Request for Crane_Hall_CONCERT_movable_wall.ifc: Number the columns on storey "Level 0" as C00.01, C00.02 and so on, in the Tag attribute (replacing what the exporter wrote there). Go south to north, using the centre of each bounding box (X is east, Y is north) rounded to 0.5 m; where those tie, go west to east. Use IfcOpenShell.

First a look at what the model holds.

```python
import ifcopenshell
import ifcopenshell.util.element
import ifcopenshell.util.placement

model = ifcopenshell.open("Crane_Hall_CONCERT_movable_wall.ifc")
print(model.schema)
storey = next(s for s in model.by_type("IfcBuildingStorey") if s.Name == "Level 0")
columns = [e for e in ifcopenshell.util.element.get_decomposition(storey) if e.is_a("IfcColumn")]
for e in sorted(columns, key=lambda e: e.id()):
    origin = ifcopenshell.util.placement.get_local_placement(e.ObjectPlacement)[:3, 3]
    print(e.id(), e.Tag, e.Name, origin.round(2) + 0.0, sep=" | ")
```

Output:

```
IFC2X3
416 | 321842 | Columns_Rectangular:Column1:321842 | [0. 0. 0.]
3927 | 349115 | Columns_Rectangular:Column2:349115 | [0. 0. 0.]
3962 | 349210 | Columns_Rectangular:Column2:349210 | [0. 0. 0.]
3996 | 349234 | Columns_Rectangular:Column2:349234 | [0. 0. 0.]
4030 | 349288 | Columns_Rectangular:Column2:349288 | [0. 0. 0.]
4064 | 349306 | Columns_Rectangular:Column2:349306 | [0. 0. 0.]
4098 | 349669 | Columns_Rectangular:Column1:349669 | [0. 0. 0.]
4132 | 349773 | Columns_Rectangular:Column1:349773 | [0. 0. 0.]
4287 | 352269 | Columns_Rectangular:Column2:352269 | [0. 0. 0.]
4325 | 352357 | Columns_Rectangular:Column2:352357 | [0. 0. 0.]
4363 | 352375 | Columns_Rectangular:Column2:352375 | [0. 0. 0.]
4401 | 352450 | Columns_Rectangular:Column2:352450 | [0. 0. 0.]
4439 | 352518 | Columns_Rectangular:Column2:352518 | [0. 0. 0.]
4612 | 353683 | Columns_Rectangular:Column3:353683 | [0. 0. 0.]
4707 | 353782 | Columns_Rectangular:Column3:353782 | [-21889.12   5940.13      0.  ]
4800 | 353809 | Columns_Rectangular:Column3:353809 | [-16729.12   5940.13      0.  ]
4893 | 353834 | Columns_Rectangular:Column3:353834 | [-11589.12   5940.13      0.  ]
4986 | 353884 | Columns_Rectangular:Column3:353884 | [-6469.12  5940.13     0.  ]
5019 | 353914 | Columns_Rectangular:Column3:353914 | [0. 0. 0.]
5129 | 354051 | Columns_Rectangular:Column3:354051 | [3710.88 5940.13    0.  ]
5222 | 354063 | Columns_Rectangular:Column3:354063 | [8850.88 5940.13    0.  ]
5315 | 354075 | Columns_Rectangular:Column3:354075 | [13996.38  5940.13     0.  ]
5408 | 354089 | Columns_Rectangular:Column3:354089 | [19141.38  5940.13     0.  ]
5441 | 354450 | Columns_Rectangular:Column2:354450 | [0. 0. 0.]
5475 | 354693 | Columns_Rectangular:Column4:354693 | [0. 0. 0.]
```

```python
import ifcopenshell
import ifcopenshell.geom
import ifcopenshell.util.element
import ifcopenshell.util.shape

model = ifcopenshell.open("Crane_Hall_CONCERT_movable_wall.ifc")
settings = ifcopenshell.geom.settings()
settings.set("use-world-coords", True)


def centre(element):
    shape = ifcopenshell.geom.create_shape(settings, element)
    return ifcopenshell.util.shape.get_bbox_centroid(shape.geometry)


storey = next(s for s in model.by_type("IfcBuildingStorey") if s.Name == "Level 0")
columns = [e for e in ifcopenshell.util.element.get_decomposition(storey) if e.is_a("IfcColumn")]

# Insertion points can sit at a corner or the storey origin, so sort by the geometry (in metres).
centres = {e: centre(e) for e in columns}
columns.sort(key=lambda e: (round(centres[e][1] / 0.5), centres[e][0]))

for i, e in enumerate(columns, start=1):
    number = f"C00.{i:02d}"
    e.Tag = number
    print(e.id(), number)

model.write("Crane_Hall_CONCERT_movable_wall_v2.ifc")
```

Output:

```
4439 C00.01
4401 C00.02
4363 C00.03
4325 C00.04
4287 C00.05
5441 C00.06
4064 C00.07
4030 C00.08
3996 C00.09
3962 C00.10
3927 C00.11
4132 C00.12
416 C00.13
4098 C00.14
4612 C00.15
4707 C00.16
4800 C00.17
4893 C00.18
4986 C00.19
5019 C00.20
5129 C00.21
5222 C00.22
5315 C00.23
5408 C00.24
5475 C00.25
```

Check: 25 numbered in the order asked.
